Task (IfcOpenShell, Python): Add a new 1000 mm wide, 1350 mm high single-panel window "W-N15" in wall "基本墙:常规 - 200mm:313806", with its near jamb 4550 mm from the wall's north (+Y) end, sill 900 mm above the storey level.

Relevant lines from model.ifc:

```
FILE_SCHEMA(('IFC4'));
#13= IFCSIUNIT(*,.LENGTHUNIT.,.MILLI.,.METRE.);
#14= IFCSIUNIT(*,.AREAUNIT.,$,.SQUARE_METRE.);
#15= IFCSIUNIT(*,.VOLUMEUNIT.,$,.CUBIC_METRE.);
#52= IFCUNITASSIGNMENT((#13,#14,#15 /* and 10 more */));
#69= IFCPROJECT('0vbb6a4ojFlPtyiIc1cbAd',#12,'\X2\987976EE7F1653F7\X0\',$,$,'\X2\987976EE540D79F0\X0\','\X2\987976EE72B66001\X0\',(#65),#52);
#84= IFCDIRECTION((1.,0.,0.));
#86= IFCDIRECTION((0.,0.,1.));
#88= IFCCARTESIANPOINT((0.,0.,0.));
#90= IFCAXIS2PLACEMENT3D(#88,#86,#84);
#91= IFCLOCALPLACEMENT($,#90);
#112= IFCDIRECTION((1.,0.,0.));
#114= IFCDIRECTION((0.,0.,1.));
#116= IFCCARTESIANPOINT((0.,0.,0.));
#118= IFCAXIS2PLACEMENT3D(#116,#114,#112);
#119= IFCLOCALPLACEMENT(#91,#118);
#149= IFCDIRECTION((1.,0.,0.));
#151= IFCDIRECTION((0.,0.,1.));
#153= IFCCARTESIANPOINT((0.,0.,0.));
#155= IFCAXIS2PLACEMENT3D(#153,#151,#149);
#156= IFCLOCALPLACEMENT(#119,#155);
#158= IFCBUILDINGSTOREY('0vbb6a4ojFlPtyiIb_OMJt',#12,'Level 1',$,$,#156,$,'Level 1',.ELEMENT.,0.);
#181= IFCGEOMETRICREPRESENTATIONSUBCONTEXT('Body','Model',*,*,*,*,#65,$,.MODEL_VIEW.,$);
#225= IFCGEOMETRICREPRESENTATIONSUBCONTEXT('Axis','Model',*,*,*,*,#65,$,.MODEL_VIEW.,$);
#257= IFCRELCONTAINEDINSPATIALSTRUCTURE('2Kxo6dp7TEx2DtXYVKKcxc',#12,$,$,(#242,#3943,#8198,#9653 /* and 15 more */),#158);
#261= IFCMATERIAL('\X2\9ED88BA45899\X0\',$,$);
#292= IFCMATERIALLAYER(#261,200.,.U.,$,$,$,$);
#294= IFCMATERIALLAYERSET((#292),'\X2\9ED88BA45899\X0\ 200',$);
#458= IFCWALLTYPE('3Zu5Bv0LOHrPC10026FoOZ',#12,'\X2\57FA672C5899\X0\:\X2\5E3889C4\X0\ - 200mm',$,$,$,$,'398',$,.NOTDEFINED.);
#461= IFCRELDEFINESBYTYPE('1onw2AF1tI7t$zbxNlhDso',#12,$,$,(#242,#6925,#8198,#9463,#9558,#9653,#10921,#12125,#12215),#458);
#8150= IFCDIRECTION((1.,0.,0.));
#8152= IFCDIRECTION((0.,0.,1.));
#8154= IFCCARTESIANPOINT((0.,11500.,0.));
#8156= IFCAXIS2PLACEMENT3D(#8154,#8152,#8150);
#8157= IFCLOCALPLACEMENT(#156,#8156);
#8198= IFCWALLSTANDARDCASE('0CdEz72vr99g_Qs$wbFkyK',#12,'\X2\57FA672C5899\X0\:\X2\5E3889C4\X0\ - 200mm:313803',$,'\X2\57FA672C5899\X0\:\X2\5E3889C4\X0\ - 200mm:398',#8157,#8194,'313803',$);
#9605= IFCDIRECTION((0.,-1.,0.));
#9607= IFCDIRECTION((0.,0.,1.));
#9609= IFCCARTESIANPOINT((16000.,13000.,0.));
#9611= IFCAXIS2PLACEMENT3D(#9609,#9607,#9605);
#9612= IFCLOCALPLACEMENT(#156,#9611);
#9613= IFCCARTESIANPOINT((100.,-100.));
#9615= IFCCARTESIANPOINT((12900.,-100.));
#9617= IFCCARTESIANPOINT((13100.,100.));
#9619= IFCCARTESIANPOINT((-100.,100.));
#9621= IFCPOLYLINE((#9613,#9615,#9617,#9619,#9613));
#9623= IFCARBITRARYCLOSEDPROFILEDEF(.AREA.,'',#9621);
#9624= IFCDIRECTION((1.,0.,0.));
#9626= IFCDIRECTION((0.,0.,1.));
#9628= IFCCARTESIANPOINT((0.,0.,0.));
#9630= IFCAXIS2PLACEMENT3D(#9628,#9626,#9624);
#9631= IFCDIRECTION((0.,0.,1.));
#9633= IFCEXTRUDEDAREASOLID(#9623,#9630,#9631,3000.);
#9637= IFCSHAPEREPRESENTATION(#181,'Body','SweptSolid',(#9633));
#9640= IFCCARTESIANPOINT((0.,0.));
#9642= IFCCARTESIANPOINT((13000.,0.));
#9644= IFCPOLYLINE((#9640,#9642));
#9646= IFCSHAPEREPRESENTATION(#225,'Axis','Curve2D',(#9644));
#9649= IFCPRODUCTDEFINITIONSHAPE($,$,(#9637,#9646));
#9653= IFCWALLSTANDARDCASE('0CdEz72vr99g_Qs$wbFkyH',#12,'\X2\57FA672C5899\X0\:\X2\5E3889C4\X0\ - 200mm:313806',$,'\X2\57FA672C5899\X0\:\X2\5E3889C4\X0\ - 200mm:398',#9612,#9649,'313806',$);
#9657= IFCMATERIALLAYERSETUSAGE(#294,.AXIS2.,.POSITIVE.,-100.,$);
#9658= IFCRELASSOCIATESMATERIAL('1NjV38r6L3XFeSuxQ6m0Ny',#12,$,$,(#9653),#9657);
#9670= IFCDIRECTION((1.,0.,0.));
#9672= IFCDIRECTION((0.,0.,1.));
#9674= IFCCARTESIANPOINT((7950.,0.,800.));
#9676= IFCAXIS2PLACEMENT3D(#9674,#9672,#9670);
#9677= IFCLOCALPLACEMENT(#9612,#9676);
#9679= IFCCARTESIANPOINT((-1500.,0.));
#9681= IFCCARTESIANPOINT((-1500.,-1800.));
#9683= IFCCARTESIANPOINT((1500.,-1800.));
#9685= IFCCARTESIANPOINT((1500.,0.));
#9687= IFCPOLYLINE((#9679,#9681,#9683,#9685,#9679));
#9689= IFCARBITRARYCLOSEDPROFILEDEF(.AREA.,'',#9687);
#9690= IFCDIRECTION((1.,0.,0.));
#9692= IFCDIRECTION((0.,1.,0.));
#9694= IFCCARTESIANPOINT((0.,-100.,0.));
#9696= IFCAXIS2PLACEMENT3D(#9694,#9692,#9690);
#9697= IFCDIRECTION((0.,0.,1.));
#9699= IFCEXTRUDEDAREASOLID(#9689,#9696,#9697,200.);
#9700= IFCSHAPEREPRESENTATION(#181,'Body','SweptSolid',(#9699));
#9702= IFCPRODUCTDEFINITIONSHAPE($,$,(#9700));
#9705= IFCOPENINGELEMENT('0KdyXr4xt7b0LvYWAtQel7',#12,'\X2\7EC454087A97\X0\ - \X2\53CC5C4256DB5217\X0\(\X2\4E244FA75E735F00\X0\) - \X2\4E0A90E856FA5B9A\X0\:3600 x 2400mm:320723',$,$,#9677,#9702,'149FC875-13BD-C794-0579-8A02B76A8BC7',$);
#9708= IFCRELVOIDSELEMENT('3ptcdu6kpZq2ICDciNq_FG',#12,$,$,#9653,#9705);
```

```python
import numpy as np
import ifcopenshell
import ifcopenshell.api.feature
import ifcopenshell.api.geometry
import ifcopenshell.api.root
import ifcopenshell.api.spatial
import ifcopenshell.geom
import ifcopenshell.util.element
import ifcopenshell.util.placement
import ifcopenshell.util.representation
import ifcopenshell.util.shape
import ifcopenshell.util.unit

model = ifcopenshell.open("model.ifc")
unit_scale = ifcopenshell.util.unit.calculate_unit_scale(model)
settings = ifcopenshell.geom.settings()


def volume(element):
    """Net volume in cubic metres, openings subtracted."""
    shape = ifcopenshell.geom.create_shape(settings, element)
    return ifcopenshell.util.shape.get_volume(shape.geometry)


wall = model.by_guid("0CdEz72vr99g_Qs$wbFkyH")
storey = ifcopenshell.util.element.get_container(wall, ifc_class="IfcBuildingStorey")
context = ifcopenshell.util.representation.get_context(model, "Model", "Body", "MODEL_VIEW")
before = volume(wall)

width, height, from_end, sill = 1, 1.35, 4.55, 0.9  # metres

# The wall runs along its own X axis, and the end named is its -X end.
wall_shape = ifcopenshell.geom.create_shape(settings, wall)
x, y, z = ifcopenshell.util.shape.get_vertices(wall_shape.geometry).T
start = x.min() + from_end
face, thickness = float(y.min()), float(y.max() - y.min())
wall_matrix = ifcopenshell.util.placement.get_local_placement(wall.ObjectPlacement)
level = ifcopenshell.util.placement.get_local_placement(storey.ObjectPlacement)[2, 3]


def in_wall(x, y):
    """Placement at x, y metres in the wall's axes, at sill height."""
    matrix = wall_matrix.copy()
    matrix[:, 3] = wall_matrix @ np.array([x / unit_scale, y / unit_scale, 0.0, 1.0])
    matrix[2, 3] = level + sill / unit_scale
    return matrix


# Opening: a box that overshoots both wall faces by 50 mm.
opening = ifcopenshell.api.root.create_entity(model, ifc_class="IfcOpeningElement", predefined_type="OPENING")
box = ifcopenshell.api.geometry.add_wall_representation(
    model, context=context, length=width, height=height, thickness=thickness + 0.1
)
ifcopenshell.api.geometry.assign_representation(model, product=opening, representation=box)
ifcopenshell.api.geometry.edit_object_placement(model, product=opening, matrix=in_wall(start, face - 0.05), is_si=False)
ifcopenshell.api.feature.add_feature(model, feature=opening, element=wall)

window = ifcopenshell.api.root.create_entity(model, ifc_class="IfcWindow", name="W-N15", predefined_type="WINDOW")
window.OverallWidth, window.OverallHeight = width / unit_scale, height / unit_scale
window.PartitioningType = "SINGLE_PANEL"
body = ifcopenshell.api.geometry.add_window_representation(
    model,
    context=context,
    overall_width=window.OverallWidth,
    overall_height=window.OverallHeight,
    partition_type="SINGLE_PANEL",
)
ifcopenshell.api.geometry.assign_representation(model, product=window, representation=body)
ifcopenshell.api.spatial.assign_container(model, products=[window], relating_structure=storey)
ifcopenshell.api.feature.add_filling(model, opening=opening, element=window)

# Centre the window in the wall's thickness.
ifcopenshell.api.geometry.edit_object_placement(model, product=window, matrix=in_wall(start, face), is_si=False)
window_shape = ifcopenshell.geom.create_shape(settings, window)
depth = ifcopenshell.util.shape.get_vertices(window_shape.geometry)[:, 1]
offset = face + thickness / 2 - (depth.min() + depth.max()) / 2
ifcopenshell.api.geometry.edit_object_placement(model, product=window, matrix=in_wall(start, offset), is_si=False)

after = volume(wall)

print(f"wall volume {before:.3f} -> {after:.3f} m3")

model.write("model_edited.ifc")
```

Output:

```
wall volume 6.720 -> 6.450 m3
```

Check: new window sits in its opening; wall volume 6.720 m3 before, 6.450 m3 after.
